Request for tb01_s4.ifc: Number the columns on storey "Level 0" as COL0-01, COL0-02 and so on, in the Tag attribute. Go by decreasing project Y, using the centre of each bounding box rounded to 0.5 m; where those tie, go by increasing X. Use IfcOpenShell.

First a look at what the model holds.

```python
import ifcopenshell
import ifcopenshell.util.element
import ifcopenshell.util.placement

model = ifcopenshell.open("tb01_s4.ifc")
print(model.schema)
storey = next(s for s in model.by_type("IfcBuildingStorey") if s.Name == "Level 0")
columns = [e for e in ifcopenshell.util.element.get_decomposition(storey) if e.is_a("IfcColumn")]
for e in sorted(columns, key=lambda e: e.id()):
    origin = ifcopenshell.util.placement.get_local_placement(e.ObjectPlacement)[:3, 3]
    print(e.id(), e.Tag, e.Name, origin.round(2) + 0.0, sep=" | ")
```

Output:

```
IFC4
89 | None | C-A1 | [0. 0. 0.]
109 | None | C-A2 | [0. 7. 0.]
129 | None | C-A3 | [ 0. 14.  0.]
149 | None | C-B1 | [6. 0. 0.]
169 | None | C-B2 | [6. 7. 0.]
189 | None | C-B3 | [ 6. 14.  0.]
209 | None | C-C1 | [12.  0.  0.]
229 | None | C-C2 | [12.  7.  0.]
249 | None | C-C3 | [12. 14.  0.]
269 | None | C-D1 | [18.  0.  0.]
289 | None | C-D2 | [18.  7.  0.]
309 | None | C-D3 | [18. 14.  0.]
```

```python
import ifcopenshell
import ifcopenshell.geom
import ifcopenshell.util.element
import ifcopenshell.util.shape

model = ifcopenshell.open("tb01_s4.ifc")
settings = ifcopenshell.geom.settings()
settings.set("use-world-coords", True)


def centre(element):
    shape = ifcopenshell.geom.create_shape(settings, element)
    return ifcopenshell.util.shape.get_bbox_centroid(shape.geometry)


storey = next(s for s in model.by_type("IfcBuildingStorey") if s.Name == "Level 0")
columns = [e for e in ifcopenshell.util.element.get_decomposition(storey) if e.is_a("IfcColumn")]

# Insertion points can sit at a corner or the storey origin, so sort by the geometry (in metres).
centres = {e: centre(e) for e in columns}
columns.sort(key=lambda e: (-round(centres[e][1] / 0.5), centres[e][0]))

for i, e in enumerate(columns, start=1):
    number = f"COL0-{i:02d}"
    e.Tag = number
    print(e.id(), number)

model.write("tb01_s4_updated.ifc")
```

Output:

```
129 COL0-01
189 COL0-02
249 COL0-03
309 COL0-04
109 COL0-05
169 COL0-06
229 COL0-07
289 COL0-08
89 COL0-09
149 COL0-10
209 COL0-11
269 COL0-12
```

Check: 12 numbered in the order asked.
